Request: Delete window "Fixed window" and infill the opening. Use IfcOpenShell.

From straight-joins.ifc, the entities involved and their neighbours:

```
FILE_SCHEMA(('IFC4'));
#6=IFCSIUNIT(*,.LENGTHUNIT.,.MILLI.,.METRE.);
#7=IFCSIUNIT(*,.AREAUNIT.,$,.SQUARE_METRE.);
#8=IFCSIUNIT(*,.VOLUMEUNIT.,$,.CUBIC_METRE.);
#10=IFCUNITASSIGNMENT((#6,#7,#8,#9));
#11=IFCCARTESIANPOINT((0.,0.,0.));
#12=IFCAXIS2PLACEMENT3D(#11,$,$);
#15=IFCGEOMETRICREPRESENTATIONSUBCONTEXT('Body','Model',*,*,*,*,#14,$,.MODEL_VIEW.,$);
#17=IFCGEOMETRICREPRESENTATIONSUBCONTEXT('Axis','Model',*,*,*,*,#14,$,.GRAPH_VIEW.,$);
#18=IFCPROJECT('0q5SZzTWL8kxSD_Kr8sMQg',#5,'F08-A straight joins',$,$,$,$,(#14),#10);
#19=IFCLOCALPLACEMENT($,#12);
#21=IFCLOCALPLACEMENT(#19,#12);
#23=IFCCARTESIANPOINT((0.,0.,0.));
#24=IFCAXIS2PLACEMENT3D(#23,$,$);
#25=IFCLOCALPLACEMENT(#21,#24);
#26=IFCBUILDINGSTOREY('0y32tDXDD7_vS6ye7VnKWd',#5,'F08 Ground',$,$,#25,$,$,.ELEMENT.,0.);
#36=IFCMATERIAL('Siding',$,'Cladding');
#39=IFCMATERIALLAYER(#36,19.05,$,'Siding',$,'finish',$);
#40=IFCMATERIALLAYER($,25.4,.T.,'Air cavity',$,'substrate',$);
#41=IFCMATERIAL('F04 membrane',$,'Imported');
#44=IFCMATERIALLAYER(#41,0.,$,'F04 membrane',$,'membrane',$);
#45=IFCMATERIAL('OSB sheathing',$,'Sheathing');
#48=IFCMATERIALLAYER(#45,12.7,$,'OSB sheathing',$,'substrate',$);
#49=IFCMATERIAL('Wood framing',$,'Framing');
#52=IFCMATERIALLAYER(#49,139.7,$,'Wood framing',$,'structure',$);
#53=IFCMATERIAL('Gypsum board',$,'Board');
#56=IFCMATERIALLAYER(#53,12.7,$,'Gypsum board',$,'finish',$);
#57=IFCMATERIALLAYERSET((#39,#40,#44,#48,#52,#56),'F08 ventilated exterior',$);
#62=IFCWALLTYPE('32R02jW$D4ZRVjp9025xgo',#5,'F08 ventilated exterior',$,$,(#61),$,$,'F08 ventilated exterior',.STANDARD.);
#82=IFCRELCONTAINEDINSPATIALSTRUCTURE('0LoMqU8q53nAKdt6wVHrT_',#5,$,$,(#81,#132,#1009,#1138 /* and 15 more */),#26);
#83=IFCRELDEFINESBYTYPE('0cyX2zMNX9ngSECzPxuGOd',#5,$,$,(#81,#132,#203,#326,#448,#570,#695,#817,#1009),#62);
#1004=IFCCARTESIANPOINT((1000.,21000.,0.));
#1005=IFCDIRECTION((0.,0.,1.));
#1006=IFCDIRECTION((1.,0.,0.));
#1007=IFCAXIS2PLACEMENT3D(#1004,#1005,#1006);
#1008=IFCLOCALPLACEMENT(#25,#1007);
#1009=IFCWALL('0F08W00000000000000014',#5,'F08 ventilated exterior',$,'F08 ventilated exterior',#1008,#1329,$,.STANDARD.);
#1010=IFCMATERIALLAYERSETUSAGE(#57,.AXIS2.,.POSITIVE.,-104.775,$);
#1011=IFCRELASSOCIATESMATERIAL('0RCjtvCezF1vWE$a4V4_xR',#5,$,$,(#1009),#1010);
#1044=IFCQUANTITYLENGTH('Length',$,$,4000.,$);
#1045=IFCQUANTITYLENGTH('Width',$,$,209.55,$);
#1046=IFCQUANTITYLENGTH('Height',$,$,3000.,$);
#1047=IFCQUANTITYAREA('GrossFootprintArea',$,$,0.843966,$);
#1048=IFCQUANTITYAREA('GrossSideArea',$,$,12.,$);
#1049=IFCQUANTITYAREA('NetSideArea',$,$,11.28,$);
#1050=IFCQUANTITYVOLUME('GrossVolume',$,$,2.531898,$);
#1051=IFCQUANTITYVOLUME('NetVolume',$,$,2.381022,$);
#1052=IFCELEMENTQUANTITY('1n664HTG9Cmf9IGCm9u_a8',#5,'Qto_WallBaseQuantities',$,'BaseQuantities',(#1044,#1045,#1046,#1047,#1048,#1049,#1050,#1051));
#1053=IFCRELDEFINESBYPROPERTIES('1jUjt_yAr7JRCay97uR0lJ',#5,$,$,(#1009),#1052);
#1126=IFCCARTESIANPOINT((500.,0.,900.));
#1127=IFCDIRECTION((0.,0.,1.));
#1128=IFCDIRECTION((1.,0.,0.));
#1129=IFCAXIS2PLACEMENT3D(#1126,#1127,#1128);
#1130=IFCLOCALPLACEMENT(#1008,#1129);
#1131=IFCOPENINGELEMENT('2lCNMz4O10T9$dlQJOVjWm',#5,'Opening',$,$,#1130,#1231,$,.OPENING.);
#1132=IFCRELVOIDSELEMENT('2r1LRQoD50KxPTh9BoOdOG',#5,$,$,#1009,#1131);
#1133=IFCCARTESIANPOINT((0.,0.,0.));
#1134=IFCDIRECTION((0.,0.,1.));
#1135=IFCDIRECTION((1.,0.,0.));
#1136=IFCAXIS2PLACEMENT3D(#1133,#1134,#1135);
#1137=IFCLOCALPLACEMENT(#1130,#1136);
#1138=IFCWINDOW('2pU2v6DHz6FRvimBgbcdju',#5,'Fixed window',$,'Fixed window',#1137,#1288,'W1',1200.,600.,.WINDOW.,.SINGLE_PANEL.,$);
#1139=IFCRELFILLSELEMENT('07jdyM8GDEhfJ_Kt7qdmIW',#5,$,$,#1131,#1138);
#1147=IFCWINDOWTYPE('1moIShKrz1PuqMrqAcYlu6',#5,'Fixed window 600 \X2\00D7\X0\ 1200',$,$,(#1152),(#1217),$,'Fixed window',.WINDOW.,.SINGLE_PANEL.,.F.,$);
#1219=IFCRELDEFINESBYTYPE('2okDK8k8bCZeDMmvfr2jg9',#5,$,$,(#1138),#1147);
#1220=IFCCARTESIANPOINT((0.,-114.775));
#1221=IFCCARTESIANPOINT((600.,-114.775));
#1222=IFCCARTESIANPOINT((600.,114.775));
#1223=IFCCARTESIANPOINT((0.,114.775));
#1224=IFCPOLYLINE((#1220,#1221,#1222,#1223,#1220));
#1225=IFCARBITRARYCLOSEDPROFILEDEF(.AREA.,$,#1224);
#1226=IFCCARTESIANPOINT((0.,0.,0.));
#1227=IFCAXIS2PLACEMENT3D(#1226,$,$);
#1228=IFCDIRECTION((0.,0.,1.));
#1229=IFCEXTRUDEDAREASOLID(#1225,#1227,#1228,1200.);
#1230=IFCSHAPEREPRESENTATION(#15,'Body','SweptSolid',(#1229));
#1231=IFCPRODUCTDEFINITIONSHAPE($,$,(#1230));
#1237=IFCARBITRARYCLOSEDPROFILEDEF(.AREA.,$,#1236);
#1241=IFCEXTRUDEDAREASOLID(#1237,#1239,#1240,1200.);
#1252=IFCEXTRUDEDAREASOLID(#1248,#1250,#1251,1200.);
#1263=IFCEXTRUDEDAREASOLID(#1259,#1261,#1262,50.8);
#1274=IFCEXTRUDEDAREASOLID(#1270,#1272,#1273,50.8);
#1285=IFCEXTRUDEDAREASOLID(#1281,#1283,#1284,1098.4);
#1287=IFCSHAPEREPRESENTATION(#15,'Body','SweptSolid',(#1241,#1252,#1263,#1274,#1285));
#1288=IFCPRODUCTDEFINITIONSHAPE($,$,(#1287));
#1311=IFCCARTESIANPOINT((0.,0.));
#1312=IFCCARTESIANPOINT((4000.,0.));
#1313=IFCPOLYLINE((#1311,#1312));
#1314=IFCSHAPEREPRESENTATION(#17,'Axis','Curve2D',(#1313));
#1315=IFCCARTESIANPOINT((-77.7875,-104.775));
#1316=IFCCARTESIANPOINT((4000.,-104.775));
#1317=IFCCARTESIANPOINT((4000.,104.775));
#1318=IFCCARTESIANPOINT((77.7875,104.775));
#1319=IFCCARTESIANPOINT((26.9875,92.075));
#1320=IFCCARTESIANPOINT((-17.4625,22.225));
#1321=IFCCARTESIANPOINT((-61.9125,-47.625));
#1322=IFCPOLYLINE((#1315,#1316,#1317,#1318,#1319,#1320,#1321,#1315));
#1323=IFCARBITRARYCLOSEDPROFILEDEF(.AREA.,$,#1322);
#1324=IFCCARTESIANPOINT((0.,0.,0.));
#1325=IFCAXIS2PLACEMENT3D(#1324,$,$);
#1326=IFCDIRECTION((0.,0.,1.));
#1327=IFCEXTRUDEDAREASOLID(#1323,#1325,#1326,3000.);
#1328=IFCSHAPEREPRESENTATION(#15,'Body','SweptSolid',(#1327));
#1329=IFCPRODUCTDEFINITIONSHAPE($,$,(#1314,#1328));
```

```python
import ifcopenshell
import ifcopenshell.api.feature
import ifcopenshell.api.pset
import ifcopenshell.api.root
import ifcopenshell.geom
import ifcopenshell.util.element
import ifcopenshell.util.shape
import ifcopenshell.util.unit

model = ifcopenshell.open("straight-joins.ifc")
area_scale = ifcopenshell.util.unit.calculate_unit_scale(model, "AREAUNIT")
volume_scale = ifcopenshell.util.unit.calculate_unit_scale(model, "VOLUMEUNIT")
settings = ifcopenshell.geom.settings()


def volume(element):
    """Net volume in cubic metres, openings subtracted."""
    shape = ifcopenshell.geom.create_shape(settings, element)
    return ifcopenshell.util.shape.get_volume(shape.geometry)


window = model.by_guid("2pU2v6DHz6FRvimBgbcdju")
opening = window.FillsVoids[0].RelatingOpeningElement
wall = opening.VoidsElements[0].RelatingBuildingElement
before = volume(wall)

ifcopenshell.api.root.remove_product(model, product=window)
ifcopenshell.api.feature.remove_feature(model, feature=opening)

after = volume(wall)
thickness = 0.2096  # wall thickness in metres

# Update the wall's stored quantities.
qto = model.by_id(ifcopenshell.util.element.get_pset(wall, "Qto_WallBaseQuantities", should_inherit=False)["id"])
ifcopenshell.api.pset.edit_qto(model, qto=qto, properties={
    "NetSideArea": after / thickness / area_scale,
    "NetVolume": after / volume_scale,
})

print(f"wall volume {before:.3f} -> {after:.3f} m3")

model.write("straight-joins_v2.ifc")
```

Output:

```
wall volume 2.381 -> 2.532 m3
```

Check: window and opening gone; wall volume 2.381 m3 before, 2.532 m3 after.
